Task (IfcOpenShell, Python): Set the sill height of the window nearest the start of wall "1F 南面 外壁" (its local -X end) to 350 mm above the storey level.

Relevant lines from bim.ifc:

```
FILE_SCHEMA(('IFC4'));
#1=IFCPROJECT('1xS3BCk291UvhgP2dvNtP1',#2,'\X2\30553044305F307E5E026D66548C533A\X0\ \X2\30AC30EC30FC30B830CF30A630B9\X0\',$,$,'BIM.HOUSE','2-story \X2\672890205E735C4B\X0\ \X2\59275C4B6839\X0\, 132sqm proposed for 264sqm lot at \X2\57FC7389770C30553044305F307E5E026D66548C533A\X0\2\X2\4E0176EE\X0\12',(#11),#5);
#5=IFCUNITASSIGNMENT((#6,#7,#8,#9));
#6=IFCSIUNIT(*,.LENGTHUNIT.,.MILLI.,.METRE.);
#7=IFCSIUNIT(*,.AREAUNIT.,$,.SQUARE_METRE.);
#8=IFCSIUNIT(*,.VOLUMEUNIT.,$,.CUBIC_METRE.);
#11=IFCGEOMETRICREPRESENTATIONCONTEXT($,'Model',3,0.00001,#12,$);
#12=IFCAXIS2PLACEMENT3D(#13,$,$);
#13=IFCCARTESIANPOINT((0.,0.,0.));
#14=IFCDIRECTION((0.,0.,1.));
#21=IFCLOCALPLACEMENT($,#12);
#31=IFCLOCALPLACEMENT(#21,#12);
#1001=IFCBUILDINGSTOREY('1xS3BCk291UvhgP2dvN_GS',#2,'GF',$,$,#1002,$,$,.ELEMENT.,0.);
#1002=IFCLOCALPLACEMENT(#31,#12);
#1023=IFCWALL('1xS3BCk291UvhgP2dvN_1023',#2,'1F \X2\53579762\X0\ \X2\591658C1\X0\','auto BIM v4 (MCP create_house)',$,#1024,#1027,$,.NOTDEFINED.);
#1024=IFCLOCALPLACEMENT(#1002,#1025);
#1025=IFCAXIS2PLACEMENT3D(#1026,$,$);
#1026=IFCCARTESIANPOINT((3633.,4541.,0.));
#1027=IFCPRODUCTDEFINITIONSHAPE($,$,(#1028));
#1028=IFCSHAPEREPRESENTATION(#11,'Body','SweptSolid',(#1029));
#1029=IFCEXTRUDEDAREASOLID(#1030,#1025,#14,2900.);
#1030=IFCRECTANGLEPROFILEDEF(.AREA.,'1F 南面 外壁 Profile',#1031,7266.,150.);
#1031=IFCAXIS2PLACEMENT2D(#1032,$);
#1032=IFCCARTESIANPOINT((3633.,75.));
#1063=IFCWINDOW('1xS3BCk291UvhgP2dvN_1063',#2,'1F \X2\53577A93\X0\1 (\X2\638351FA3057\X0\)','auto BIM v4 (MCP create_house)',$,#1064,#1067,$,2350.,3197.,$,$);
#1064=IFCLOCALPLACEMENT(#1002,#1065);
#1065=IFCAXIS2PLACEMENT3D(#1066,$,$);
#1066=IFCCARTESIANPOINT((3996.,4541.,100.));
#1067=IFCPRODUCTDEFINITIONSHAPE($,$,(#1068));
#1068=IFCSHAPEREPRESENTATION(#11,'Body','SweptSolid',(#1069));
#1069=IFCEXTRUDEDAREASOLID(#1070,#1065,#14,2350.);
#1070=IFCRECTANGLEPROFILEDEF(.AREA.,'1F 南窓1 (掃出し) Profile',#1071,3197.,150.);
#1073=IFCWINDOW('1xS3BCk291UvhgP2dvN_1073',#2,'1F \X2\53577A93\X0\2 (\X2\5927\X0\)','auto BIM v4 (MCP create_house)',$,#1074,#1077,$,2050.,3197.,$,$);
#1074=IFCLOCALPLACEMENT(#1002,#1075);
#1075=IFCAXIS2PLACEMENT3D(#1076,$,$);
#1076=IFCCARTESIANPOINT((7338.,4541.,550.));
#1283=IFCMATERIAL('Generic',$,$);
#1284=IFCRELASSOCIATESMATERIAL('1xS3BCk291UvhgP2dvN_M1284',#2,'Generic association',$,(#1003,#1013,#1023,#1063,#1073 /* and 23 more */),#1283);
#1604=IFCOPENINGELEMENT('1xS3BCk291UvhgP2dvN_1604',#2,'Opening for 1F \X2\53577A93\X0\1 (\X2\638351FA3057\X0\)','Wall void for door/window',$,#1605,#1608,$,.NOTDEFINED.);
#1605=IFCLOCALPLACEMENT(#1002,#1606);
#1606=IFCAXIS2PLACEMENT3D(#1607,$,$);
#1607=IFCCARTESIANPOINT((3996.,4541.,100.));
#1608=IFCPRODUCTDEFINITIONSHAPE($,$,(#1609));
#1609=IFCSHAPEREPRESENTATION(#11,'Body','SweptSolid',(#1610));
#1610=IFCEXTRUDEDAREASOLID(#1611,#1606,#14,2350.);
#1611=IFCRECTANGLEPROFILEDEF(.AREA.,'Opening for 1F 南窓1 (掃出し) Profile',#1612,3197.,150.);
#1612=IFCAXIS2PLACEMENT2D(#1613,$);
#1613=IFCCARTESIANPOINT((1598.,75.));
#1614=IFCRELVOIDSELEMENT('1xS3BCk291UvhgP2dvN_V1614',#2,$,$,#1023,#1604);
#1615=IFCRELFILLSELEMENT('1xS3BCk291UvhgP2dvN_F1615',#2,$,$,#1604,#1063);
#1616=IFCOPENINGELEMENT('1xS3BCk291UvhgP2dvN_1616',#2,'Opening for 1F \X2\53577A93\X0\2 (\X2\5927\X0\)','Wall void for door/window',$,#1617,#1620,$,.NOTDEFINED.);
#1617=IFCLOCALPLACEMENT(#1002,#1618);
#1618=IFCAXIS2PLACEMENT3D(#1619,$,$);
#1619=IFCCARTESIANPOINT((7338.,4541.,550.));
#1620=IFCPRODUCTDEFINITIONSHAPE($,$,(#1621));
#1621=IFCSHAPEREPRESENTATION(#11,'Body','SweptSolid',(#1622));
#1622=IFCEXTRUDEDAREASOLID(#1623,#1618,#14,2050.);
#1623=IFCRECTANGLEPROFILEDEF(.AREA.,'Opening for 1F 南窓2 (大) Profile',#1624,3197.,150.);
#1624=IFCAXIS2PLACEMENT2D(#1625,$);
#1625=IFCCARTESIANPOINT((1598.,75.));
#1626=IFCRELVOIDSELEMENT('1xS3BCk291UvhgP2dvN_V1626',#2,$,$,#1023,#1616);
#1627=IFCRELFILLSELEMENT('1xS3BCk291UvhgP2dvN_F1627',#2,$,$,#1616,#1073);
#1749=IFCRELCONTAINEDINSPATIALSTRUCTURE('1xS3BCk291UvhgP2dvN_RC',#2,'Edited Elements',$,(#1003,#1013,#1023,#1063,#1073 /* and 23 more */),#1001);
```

```python
import numpy as np
import ifcopenshell
import ifcopenshell.api.geometry
import ifcopenshell.geom
import ifcopenshell.util.element
import ifcopenshell.util.placement
import ifcopenshell.util.shape
import ifcopenshell.util.unit

model = ifcopenshell.open("bim.ifc")
unit_scale = ifcopenshell.util.unit.calculate_unit_scale(model)

window = model.by_id(1063)
opening = window.FillsVoids[0].RelatingOpeningElement
storey = ifcopenshell.util.element.get_container(window, ifc_class="IfcBuildingStorey")
level = ifcopenshell.util.placement.get_local_placement(storey.ObjectPlacement)[2, 3]

# The opening's origin need not be at the sill, so measure its lowest point.
shape = ifcopenshell.geom.create_shape(ifcopenshell.geom.settings(), opening)
bottom = ifcopenshell.util.shape.get_shape_bottom_elevation(shape, shape.geometry) / unit_scale
dz = level + 0.35 / unit_scale - bottom

shift = np.array([0.0, 0.0, dz])
# The window is not placed relative to its opening, so move both.
for product in (opening, window):
    matrix = ifcopenshell.util.placement.get_local_placement(product.ObjectPlacement)
    matrix[:3, 3] += shift
    ifcopenshell.api.geometry.edit_object_placement(model, product=product, matrix=matrix, is_si=False)

print(f"moved by {dz * unit_scale:+.3f} m")

model.write("bim_updated.ifc")
```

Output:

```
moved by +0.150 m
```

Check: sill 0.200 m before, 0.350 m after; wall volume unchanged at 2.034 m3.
